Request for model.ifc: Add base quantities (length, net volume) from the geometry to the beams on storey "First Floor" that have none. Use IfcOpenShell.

First a look at what the model holds.

```python
import ifcopenshell
import ifcopenshell.util.element
import ifcopenshell.util.unit

model = ifcopenshell.open("model.ifc")
print(model.schema)
for unit_type in ("LENGTHUNIT", "AREAUNIT", "VOLUMEUNIT"):
    print(unit_type, ifcopenshell.util.unit.calculate_unit_scale(model, unit_type))
storey = next(s for s in model.by_type("IfcBuildingStorey") if s.Name == "First Floor")
beams = [e for e in ifcopenshell.util.element.get_decomposition(storey) if e.is_a("IfcBeam")]
for e in sorted(beams, key=lambda e: e.id()):
    print(e.id(), e.is_a(), e.Name, list(ifcopenshell.util.element.get_psets(e, qtos_only=True)), sep=" | ")
```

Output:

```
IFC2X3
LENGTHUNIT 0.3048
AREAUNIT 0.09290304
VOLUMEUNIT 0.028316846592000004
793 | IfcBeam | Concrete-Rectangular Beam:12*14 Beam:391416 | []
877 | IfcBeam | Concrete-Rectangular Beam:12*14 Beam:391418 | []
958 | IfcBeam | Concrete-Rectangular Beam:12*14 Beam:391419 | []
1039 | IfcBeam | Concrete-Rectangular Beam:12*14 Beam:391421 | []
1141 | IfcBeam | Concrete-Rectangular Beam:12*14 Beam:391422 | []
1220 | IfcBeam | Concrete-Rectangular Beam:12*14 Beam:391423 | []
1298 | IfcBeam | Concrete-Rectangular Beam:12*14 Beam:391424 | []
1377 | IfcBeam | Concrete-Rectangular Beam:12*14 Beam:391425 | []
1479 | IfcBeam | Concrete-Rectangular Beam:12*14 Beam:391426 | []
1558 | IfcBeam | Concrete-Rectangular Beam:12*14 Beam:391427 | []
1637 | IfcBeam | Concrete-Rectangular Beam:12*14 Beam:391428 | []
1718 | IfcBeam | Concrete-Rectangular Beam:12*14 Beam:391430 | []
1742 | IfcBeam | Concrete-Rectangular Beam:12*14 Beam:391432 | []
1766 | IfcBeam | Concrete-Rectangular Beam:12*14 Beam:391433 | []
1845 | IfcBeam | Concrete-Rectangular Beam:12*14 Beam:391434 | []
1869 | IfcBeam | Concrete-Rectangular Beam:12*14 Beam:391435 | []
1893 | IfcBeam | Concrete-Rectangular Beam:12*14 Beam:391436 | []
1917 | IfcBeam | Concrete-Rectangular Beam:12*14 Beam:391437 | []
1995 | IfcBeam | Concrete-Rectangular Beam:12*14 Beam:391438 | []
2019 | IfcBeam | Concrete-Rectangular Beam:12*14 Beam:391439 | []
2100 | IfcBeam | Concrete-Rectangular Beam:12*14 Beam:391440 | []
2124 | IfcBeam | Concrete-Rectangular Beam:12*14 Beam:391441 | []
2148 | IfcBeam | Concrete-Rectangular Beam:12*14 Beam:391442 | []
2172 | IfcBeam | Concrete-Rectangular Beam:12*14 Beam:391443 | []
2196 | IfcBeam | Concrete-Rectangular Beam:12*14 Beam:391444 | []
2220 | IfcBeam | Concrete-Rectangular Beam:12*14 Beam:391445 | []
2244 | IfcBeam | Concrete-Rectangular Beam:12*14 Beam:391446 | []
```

```python
import ifcopenshell
import ifcopenshell.api.pset
import ifcopenshell.geom
import ifcopenshell.util.element
import ifcopenshell.util.shape
import ifcopenshell.util.unit

model = ifcopenshell.open("model.ifc")
unit_scale = ifcopenshell.util.unit.calculate_unit_scale(model)
volume_scale = ifcopenshell.util.unit.calculate_unit_scale(model, "VOLUMEUNIT")
settings = ifcopenshell.geom.settings()

storey = next(s for s in model.by_type("IfcBuildingStorey") if s.Name == "First Floor")
beams = [e for e in ifcopenshell.util.element.get_decomposition(storey) if e.is_a("IfcBeam")]

for e in sorted(beams, key=lambda e: e.id()):
    if ifcopenshell.util.element.get_psets(e, qtos_only=True, should_inherit=False):
        continue
    # Geometry comes back in metres, in the element's own axes.
    shape = ifcopenshell.geom.create_shape(settings, e)
    values = {
        "Length": ifcopenshell.util.shape.get_max_xyz(shape.geometry) / unit_scale,
        "NetVolume": ifcopenshell.util.shape.get_volume(shape.geometry) / volume_scale,
    }
    qto = ifcopenshell.api.pset.add_qto(model, product=e, name="BaseQuantities")
    ifcopenshell.api.pset.edit_qto(model, qto=qto, properties=values)
    print(e.id(), {k: round(v, 3) for k, v in values.items()})

model.write("model-out.ifc")
```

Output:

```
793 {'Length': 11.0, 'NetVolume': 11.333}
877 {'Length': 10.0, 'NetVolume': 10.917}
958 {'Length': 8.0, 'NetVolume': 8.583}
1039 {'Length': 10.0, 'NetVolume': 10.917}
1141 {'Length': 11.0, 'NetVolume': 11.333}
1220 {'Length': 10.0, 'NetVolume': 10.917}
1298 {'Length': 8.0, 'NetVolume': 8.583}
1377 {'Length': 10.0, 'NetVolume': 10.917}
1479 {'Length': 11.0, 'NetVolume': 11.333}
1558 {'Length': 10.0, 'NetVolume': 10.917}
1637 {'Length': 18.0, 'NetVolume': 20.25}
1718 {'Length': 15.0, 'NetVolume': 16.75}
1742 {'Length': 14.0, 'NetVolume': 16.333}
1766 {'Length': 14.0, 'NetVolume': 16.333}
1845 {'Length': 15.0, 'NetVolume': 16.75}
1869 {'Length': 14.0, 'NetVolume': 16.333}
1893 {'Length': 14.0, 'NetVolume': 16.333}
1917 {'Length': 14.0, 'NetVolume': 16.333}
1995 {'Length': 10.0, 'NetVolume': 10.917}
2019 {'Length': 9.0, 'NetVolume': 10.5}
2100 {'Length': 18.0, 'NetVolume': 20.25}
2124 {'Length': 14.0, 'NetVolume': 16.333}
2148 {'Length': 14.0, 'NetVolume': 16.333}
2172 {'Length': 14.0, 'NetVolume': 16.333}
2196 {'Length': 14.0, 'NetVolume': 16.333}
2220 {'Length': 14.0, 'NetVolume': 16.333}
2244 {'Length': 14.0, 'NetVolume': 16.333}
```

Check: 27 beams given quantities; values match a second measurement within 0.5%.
